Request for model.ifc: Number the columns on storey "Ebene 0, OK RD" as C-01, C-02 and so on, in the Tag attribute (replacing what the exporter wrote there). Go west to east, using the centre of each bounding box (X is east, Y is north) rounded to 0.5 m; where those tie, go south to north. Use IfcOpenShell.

First a look at what the model holds.

```python
import ifcopenshell
import ifcopenshell.util.element
import ifcopenshell.util.placement

model = ifcopenshell.open("model.ifc")
print(model.schema)
storey = next(s for s in model.by_type("IfcBuildingStorey") if s.Name == "Ebene 0, OK RD")
columns = [e for e in ifcopenshell.util.element.get_decomposition(storey) if e.is_a("IfcColumn")]
for e in sorted(columns, key=lambda e: e.id()):
    origin = ifcopenshell.util.placement.get_local_placement(e.ObjectPlacement)[:3, 3]
    print(e.id(), e.Tag, e.Name, origin.round(2) + 0.0, sep=" | ")
```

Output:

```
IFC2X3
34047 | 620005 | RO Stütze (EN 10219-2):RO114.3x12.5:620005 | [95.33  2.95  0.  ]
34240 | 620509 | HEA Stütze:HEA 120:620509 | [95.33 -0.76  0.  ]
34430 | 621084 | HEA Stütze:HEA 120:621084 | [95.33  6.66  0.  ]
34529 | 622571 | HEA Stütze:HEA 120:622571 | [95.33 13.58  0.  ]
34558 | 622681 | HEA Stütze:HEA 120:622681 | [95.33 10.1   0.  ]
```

```python
import ifcopenshell
import ifcopenshell.geom
import ifcopenshell.util.element
import ifcopenshell.util.shape

model = ifcopenshell.open("model.ifc")
settings = ifcopenshell.geom.settings()
settings.set("use-world-coords", True)


def centre(element):
    shape = ifcopenshell.geom.create_shape(settings, element)
    return ifcopenshell.util.shape.get_bbox_centroid(shape.geometry)


storey = next(s for s in model.by_type("IfcBuildingStorey") if s.Name == "Ebene 0, OK RD")
columns = [e for e in ifcopenshell.util.element.get_decomposition(storey) if e.is_a("IfcColumn")]

# Insertion points can sit at a corner or the storey origin, so sort by the geometry (in metres).
centres = {e: centre(e) for e in columns}
columns.sort(key=lambda e: (round(centres[e][0] / 0.5), centres[e][1]))

for i, e in enumerate(columns, start=1):
    number = f"C-{i:02d}"
    e.Tag = number
    print(e.id(), number)

model.write("model_v2.ifc")
```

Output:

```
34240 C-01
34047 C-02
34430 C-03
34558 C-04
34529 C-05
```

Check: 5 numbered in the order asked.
